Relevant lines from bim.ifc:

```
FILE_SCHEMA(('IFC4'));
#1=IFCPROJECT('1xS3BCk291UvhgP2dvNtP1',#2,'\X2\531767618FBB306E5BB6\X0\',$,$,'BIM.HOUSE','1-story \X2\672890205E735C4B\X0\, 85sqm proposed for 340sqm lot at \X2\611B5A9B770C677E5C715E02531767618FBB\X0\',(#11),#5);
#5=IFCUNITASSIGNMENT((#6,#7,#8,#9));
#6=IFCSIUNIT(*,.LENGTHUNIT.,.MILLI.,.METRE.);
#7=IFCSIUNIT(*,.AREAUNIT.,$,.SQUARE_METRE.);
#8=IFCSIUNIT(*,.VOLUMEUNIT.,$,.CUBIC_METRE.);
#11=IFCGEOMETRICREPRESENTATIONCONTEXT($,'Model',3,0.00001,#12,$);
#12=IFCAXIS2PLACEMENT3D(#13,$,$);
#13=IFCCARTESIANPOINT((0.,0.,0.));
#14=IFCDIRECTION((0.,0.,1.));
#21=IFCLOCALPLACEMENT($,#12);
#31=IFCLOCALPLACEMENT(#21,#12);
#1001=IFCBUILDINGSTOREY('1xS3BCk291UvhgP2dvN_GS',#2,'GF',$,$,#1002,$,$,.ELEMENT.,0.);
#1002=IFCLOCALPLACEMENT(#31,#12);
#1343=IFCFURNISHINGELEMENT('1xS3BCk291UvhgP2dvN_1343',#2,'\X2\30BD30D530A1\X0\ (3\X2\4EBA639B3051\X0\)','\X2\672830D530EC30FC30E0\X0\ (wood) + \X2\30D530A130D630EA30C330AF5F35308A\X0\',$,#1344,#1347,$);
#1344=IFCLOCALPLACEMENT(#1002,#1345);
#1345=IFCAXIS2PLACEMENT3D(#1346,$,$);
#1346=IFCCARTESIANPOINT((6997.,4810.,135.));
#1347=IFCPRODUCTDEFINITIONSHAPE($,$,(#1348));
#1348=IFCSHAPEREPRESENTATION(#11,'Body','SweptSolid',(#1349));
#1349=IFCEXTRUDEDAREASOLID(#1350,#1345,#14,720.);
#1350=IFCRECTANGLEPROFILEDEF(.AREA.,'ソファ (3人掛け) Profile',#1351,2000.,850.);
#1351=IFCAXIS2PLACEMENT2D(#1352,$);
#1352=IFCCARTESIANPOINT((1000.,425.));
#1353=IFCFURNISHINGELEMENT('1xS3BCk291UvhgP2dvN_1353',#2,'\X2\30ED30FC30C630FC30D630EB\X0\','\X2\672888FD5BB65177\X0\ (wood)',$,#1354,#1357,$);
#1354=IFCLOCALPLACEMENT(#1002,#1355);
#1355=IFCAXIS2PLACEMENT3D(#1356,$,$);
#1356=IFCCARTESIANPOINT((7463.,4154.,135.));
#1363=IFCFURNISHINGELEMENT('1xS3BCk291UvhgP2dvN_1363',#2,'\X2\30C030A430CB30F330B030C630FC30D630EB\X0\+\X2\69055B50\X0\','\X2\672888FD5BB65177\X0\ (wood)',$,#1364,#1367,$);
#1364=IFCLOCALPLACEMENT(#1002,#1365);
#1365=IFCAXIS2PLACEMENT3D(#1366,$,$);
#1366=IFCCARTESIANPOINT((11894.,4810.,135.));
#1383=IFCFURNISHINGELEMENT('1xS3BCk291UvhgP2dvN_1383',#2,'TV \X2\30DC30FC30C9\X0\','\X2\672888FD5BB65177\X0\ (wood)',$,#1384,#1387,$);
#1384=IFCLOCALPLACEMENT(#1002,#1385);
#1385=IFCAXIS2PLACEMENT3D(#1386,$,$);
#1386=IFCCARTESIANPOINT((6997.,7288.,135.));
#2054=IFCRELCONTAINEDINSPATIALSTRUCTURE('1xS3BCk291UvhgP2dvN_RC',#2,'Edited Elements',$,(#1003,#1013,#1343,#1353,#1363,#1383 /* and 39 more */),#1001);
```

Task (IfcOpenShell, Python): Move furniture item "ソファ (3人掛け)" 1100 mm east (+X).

```python
import ifcopenshell
import ifcopenshell.api.geometry
import ifcopenshell.util.placement

model = ifcopenshell.open("bim.ifc")

item = model.by_guid("1xS3BCk291UvhgP2dvN_1343")
matrix = ifcopenshell.util.placement.get_local_placement(item.ObjectPlacement)
matrix[0, 3] += 1100.0
ifcopenshell.api.geometry.edit_object_placement(model, product=item, matrix=matrix, is_si=False)

print(ifcopenshell.util.placement.get_local_placement(item.ObjectPlacement).round(3) + 0.0)

model.write("bim_v2.ifc")
```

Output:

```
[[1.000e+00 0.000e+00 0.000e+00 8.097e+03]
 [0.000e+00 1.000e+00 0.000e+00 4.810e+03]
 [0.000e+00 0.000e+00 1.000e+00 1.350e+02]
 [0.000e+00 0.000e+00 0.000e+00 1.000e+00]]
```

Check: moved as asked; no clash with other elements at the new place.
